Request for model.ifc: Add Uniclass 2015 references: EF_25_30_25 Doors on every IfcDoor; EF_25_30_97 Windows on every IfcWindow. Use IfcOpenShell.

First a look at what the model holds.

```python
import ifcopenshell

model = ifcopenshell.open("model.ifc")
print(model.schema)
print("classifications:", [c.Name for c in model.by_type("IfcClassification")])
for ifc_class in ("IfcDoor", "IfcRoof", "IfcStair", "IfcWall", "IfcWindow"):
    print(ifc_class, len(model.by_type(ifc_class)))
```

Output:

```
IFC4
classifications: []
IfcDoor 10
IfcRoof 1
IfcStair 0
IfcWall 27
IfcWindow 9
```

```python
import ifcopenshell
import ifcopenshell.api.classification

model = ifcopenshell.open("model.ifc")

system = ifcopenshell.api.classification.add_classification(model, classification="Uniclass 2015")

codes = {
    "IfcDoor": ("EF_25_30_25", "Doors"),
    "IfcWindow": ("EF_25_30_97", "Windows"),
}
for ifc_class, (code, name) in codes.items():
    products = model.by_type(ifc_class)
    ifcopenshell.api.classification.add_reference(
        model, products=products, classification=system, identification=code, name=name
    )
    print(code, len(products))

model.write("model_rev.ifc")
```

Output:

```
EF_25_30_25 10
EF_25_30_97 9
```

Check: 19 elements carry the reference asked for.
